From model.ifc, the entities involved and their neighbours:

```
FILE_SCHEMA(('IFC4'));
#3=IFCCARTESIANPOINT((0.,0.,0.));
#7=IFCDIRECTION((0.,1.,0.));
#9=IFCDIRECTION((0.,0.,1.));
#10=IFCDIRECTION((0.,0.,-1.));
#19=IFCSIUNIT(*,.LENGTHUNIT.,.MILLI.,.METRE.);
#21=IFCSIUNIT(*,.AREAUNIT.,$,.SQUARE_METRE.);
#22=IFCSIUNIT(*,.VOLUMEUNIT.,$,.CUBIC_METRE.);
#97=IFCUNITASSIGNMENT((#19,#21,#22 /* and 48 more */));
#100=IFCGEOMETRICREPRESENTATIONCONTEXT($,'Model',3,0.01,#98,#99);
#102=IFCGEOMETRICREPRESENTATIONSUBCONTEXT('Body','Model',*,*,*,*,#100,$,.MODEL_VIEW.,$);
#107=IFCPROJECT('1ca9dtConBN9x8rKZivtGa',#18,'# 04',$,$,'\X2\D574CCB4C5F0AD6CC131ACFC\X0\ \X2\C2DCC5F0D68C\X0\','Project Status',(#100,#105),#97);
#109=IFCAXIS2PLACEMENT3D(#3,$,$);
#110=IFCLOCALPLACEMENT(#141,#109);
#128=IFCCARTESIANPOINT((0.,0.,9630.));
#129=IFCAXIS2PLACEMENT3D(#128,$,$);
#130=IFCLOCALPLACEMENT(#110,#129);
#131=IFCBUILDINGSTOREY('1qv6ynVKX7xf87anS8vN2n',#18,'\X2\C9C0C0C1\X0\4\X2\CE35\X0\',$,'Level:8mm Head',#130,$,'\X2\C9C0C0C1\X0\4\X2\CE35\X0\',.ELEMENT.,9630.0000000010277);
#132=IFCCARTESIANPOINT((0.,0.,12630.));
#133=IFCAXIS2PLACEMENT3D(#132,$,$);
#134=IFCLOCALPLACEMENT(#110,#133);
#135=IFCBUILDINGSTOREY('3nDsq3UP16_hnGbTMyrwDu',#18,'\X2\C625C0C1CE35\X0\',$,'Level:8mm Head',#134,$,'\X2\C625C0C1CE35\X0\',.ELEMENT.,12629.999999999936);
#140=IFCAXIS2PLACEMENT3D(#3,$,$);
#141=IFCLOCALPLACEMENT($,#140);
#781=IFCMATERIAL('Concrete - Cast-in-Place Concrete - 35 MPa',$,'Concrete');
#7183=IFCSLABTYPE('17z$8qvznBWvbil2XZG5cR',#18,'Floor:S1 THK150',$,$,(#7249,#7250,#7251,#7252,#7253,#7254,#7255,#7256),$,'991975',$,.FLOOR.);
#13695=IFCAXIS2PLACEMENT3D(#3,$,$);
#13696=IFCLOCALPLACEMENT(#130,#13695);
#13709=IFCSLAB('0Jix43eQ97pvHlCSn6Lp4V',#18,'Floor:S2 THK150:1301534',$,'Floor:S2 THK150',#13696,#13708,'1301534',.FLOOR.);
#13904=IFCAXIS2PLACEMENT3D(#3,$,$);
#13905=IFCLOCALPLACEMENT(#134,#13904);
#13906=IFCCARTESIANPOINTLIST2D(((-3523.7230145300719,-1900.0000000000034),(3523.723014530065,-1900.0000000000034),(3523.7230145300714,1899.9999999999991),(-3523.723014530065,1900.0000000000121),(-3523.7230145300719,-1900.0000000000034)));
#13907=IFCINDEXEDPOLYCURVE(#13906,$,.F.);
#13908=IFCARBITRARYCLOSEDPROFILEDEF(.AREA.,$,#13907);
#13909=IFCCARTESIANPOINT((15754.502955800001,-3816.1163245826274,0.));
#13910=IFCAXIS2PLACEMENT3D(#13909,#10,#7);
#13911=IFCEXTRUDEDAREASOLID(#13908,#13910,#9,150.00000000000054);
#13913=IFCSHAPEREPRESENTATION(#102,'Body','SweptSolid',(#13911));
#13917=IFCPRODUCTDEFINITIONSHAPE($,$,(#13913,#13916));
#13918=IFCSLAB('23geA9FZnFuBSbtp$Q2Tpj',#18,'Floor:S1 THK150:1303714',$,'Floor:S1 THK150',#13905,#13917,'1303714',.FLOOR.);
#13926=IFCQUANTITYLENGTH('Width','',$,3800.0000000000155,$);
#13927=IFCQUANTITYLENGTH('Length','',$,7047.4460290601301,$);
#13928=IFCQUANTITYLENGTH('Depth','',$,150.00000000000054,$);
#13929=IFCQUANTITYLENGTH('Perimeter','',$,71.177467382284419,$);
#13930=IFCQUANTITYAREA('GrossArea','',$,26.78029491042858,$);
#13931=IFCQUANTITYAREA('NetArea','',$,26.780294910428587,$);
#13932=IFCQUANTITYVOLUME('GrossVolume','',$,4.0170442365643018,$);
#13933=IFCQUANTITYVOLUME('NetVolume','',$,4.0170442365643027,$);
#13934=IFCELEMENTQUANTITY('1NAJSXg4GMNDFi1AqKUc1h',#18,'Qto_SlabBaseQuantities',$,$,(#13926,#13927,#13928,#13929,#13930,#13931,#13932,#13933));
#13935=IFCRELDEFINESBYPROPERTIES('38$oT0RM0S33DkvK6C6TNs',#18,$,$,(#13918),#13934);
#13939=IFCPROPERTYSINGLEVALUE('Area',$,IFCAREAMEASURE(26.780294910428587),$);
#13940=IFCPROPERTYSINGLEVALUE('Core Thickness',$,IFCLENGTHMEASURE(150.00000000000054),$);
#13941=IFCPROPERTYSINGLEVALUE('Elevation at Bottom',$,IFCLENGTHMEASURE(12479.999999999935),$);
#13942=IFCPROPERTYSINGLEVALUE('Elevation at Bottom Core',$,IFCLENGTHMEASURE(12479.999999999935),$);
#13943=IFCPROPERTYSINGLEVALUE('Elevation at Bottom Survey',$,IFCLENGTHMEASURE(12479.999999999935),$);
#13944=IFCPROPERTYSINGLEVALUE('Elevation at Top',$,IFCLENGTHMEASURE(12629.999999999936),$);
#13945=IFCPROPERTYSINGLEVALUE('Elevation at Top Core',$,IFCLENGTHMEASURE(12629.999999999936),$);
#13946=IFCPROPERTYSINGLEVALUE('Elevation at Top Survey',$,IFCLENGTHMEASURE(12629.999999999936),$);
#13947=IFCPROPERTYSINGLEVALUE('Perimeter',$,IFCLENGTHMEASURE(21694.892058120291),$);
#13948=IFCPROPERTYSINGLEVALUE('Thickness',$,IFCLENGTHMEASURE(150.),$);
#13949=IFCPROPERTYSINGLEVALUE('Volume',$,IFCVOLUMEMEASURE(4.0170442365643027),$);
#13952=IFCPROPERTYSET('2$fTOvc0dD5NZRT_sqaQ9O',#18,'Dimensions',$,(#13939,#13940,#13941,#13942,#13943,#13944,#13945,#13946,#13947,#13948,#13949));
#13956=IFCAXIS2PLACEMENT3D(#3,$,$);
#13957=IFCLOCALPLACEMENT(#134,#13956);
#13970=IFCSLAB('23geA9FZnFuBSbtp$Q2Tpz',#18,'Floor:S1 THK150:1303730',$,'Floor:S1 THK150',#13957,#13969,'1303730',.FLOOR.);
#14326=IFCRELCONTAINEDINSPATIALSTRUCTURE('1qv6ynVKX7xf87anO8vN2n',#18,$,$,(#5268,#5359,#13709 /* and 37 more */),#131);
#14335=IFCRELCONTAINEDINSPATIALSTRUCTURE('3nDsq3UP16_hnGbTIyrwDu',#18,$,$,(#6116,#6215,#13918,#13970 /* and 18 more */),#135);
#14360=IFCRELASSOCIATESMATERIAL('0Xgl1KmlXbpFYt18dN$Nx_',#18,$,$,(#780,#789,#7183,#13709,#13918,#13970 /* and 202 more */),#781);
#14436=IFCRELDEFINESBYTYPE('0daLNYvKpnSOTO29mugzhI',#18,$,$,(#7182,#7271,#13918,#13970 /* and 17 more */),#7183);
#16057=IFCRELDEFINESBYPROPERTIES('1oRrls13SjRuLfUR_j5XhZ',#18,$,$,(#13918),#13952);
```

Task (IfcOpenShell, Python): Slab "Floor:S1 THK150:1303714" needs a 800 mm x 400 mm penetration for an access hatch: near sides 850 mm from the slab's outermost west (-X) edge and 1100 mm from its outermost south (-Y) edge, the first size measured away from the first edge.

```python
import numpy as np
import ifcopenshell
import ifcopenshell.api.feature
import ifcopenshell.api.geometry
import ifcopenshell.api.pset
import ifcopenshell.api.root
import ifcopenshell.geom
import ifcopenshell.util.element
import ifcopenshell.util.placement
import ifcopenshell.util.representation
import ifcopenshell.util.shape
import ifcopenshell.util.unit

model = ifcopenshell.open("model.ifc")
unit_scale = ifcopenshell.util.unit.calculate_unit_scale(model)
area_scale = ifcopenshell.util.unit.calculate_unit_scale(model, "AREAUNIT")
volume_scale = ifcopenshell.util.unit.calculate_unit_scale(model, "VOLUMEUNIT")
settings = ifcopenshell.geom.settings()


def volume(element):
    """Net volume in cubic metres, openings subtracted."""
    shape = ifcopenshell.geom.create_shape(settings, element)
    return ifcopenshell.util.shape.get_volume(shape.geometry)


slab = model.by_guid("23geA9FZnFuBSbtp$Q2Tpj")
before = volume(slab)

# Extent in the slab's own axes, in metres. The edges named are its -X and -Y sides.
slab_shape = ifcopenshell.geom.create_shape(settings, slab)
vertices = ifcopenshell.util.shape.get_vertices(slab_shape.geometry)
x_min, y_min, bottom = vertices.min(axis=0)
top = vertices[:, 2].max()

opening = ifcopenshell.api.root.create_entity(model, ifc_class="IfcOpeningElement", name="Access hatch opening", predefined_type="OPENING")
context = ifcopenshell.util.representation.get_context(model, "Model", "Body", "MODEL_VIEW")
width, depth = 0.8, 0.4
outline = [(0.0, 0.0), (width, 0.0), (width, depth), (0.0, depth), (0.0, 0.0)]
# Overshoot both faces by 50 mm so the cut is clean.
shape = ifcopenshell.api.geometry.add_slab_representation(
    model, context=context, depth=top - bottom + 0.1, polyline=outline
)
ifcopenshell.api.geometry.assign_representation(model, product=opening, representation=shape)

matrix = ifcopenshell.util.placement.get_local_placement(slab.ObjectPlacement)
matrix[:, 3] = matrix @ np.append(np.array([x_min + 0.85, y_min + 1.1, bottom - 0.05]) / unit_scale, 1.0)
ifcopenshell.api.geometry.edit_object_placement(model, product=opening, matrix=matrix, is_si=False)
ifcopenshell.api.feature.add_feature(model, feature=opening, element=slab)

after = volume(slab)

# Update the slab's stored quantities.
qto = model.by_id(ifcopenshell.util.element.get_pset(slab, "Qto_SlabBaseQuantities", should_inherit=False)["id"])
ifcopenshell.api.pset.edit_qto(model, qto=qto, properties={
    "NetArea": after / (top - bottom) / area_scale,
    "NetVolume": after / volume_scale,
})
pset = model.by_id(ifcopenshell.util.element.get_pset(slab, "Dimensions", should_inherit=False)["id"])
ifcopenshell.api.pset.edit_pset(model, pset=pset, properties={
    "Area": model.create_entity("IfcAreaMeasure", after / (top - bottom) / area_scale),
    "Volume": model.create_entity("IfcVolumeMeasure", after / volume_scale),
})

print(f"slab volume {before:.3f} -> {after:.3f} m3")

model.write("model_v2.ifc")
```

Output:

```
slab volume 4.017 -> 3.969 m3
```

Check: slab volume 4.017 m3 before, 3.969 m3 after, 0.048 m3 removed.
